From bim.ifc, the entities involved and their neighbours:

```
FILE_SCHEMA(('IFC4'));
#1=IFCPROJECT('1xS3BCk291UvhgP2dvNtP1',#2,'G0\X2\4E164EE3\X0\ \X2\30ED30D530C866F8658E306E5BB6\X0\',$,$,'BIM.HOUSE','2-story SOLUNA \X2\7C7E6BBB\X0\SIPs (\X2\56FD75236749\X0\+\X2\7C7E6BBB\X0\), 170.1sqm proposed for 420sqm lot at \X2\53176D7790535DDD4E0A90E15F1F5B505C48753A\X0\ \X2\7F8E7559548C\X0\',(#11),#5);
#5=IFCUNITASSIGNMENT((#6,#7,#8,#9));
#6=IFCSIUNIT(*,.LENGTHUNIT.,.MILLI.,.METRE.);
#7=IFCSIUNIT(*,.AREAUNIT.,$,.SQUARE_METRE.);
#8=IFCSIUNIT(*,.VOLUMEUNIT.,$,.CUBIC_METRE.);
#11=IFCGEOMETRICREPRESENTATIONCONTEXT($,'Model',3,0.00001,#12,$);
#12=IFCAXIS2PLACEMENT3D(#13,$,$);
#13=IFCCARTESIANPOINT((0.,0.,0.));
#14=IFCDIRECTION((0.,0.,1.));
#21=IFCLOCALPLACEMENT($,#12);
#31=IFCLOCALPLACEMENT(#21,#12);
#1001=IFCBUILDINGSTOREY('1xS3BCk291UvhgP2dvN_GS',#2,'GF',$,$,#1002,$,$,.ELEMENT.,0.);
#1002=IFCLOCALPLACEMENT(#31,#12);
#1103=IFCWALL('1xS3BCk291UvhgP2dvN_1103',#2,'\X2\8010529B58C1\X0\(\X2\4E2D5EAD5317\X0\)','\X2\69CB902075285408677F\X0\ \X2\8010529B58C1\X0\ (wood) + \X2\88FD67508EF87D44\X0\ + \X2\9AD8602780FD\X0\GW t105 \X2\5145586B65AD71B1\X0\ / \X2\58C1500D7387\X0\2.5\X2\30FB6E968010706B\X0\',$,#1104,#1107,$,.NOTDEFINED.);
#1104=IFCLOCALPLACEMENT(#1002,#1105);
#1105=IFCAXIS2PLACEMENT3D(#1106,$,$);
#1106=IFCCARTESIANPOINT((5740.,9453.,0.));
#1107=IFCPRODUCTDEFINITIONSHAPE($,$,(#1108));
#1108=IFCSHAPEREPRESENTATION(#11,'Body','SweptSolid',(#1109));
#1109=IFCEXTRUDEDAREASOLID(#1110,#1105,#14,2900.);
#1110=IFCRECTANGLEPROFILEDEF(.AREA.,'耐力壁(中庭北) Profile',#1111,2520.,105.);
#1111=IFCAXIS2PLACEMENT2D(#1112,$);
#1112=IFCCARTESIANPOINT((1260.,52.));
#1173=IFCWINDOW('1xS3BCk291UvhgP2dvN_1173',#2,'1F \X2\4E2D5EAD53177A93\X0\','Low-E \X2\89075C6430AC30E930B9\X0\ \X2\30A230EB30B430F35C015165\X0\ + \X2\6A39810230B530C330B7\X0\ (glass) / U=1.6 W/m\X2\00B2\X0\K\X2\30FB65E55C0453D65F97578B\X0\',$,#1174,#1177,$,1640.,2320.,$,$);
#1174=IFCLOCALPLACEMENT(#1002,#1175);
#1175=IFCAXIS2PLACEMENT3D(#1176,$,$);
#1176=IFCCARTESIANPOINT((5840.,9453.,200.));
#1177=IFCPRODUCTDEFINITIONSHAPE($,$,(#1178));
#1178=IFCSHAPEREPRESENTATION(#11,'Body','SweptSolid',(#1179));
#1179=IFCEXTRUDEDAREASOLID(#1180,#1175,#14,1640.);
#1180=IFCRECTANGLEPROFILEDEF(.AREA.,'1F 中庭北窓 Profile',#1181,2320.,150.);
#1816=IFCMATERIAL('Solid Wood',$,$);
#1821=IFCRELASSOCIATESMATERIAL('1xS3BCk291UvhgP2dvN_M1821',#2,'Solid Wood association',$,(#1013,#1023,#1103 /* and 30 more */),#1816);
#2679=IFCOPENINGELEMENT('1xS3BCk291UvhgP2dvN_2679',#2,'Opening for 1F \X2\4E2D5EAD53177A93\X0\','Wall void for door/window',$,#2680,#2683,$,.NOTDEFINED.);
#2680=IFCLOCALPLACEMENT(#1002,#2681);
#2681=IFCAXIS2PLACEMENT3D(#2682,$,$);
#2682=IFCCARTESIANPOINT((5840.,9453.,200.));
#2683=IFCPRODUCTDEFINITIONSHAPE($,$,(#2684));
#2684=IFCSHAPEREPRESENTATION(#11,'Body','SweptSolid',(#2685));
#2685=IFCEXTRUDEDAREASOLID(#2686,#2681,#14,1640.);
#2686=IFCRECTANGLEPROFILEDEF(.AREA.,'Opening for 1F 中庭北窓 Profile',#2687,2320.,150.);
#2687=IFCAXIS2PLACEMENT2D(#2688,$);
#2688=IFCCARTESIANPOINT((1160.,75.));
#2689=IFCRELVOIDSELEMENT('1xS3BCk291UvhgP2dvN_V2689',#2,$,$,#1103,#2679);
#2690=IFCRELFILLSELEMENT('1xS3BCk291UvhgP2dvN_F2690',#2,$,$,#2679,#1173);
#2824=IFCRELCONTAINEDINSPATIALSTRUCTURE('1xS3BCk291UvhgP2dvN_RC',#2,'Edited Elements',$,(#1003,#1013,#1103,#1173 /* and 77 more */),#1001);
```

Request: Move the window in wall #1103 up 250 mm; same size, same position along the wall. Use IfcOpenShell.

```python
import numpy as np
import ifcopenshell
import ifcopenshell.api.geometry
import ifcopenshell.util.placement
import ifcopenshell.util.unit

model = ifcopenshell.open("bim.ifc")
unit_scale = ifcopenshell.util.unit.calculate_unit_scale(model)

window = model.by_guid("1xS3BCk291UvhgP2dvN_1173")
opening = window.FillsVoids[0].RelatingOpeningElement
dz = 0.25 / unit_scale

shift = np.array([0.0, 0.0, dz])
# The window is not placed relative to its opening, so move both.
for product in (opening, window):
    matrix = ifcopenshell.util.placement.get_local_placement(product.ObjectPlacement)
    matrix[:3, 3] += shift
    ifcopenshell.api.geometry.edit_object_placement(model, product=product, matrix=matrix, is_si=False)

print(f"moved by {dz * unit_scale:+.3f} m")

model.write("bim_edited.ifc")
```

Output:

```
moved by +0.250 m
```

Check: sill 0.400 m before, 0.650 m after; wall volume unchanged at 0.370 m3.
